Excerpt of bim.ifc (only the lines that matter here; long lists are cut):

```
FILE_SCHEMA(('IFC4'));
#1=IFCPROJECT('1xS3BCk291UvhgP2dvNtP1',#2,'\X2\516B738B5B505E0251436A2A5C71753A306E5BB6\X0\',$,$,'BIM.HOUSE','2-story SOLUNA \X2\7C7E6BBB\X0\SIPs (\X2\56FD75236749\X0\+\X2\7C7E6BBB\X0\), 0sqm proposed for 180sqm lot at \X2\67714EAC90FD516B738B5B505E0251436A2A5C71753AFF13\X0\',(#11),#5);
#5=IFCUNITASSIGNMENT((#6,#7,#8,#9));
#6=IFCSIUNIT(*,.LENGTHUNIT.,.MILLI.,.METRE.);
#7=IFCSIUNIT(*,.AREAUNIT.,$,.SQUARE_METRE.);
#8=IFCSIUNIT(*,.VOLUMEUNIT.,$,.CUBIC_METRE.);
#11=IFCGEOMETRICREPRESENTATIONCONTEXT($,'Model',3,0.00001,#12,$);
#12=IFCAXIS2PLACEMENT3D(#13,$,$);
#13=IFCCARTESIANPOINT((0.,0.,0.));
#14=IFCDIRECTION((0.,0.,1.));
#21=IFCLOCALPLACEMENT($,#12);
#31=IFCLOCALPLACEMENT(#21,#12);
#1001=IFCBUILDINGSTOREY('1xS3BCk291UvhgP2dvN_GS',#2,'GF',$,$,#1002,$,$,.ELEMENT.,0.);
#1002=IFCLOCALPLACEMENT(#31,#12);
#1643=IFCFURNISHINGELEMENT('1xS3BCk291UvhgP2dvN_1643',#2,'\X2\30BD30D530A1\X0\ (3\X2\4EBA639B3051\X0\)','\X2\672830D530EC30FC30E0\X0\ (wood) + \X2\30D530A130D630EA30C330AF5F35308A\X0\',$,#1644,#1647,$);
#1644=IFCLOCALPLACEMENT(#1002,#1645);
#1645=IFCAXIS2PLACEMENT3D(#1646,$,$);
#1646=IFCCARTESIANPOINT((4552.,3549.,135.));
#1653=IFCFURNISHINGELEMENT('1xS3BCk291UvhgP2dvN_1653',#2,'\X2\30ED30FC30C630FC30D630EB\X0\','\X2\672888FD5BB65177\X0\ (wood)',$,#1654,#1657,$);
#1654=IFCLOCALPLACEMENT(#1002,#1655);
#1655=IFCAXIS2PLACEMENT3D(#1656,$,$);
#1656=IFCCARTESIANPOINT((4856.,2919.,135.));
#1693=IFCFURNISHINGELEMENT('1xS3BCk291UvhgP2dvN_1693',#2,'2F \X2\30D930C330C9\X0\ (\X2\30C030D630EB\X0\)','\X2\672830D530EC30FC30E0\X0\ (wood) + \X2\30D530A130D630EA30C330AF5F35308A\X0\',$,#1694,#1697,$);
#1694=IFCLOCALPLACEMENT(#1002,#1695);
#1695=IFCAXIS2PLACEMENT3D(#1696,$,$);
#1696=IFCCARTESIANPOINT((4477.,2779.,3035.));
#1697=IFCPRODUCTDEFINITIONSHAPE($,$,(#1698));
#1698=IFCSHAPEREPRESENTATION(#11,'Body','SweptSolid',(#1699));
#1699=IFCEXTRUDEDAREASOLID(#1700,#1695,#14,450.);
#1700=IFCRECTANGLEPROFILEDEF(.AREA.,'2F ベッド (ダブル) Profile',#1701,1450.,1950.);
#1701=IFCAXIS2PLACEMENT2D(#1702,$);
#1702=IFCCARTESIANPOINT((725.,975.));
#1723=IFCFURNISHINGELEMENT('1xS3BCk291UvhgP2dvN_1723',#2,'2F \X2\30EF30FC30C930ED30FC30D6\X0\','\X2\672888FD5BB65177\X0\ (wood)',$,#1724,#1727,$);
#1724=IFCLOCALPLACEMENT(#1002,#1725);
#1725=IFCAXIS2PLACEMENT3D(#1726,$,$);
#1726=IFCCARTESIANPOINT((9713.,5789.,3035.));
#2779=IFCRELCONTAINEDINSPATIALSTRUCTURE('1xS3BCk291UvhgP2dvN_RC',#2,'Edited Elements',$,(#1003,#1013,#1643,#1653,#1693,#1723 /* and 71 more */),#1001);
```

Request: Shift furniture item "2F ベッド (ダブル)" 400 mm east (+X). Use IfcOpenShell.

```python
import ifcopenshell
import ifcopenshell.api.geometry
import ifcopenshell.util.placement
import ifcopenshell.util.unit

model = ifcopenshell.open("bim.ifc")
unit_scale = ifcopenshell.util.unit.calculate_unit_scale(model)

item = model.by_id(1693)
matrix = ifcopenshell.util.placement.get_local_placement(item.ObjectPlacement)
matrix[0, 3] += 0.4 / unit_scale
ifcopenshell.api.geometry.edit_object_placement(model, product=item, matrix=matrix, is_si=False)

print(ifcopenshell.util.placement.get_local_placement(item.ObjectPlacement).round(3) + 0.0)

model.write("bim_edited.ifc")
```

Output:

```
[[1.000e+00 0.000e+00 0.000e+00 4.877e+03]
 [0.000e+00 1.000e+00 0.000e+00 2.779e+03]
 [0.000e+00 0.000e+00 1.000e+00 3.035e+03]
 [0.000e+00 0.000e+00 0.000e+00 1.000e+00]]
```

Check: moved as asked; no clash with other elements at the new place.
